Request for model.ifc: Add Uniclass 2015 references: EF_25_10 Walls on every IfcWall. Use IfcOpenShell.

First a look at what the model holds.

```python
import ifcopenshell

model = ifcopenshell.open("model.ifc")
print(model.schema)
print("classifications:", [c.Name for c in model.by_type("IfcClassification")])
for ifc_class in ("IfcDoor", "IfcRoof", "IfcStair", "IfcWall", "IfcWindow"):
    print(ifc_class, len(model.by_type(ifc_class)))
```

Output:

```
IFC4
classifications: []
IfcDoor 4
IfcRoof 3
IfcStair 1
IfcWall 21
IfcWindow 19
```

```python
import ifcopenshell
import ifcopenshell.api.classification

model = ifcopenshell.open("model.ifc")

system = ifcopenshell.api.classification.add_classification(model, classification="Uniclass 2015")

codes = {
    "IfcWall": ("EF_25_10", "Walls"),
}
for ifc_class, (code, name) in codes.items():
    products = model.by_type(ifc_class)
    ifcopenshell.api.classification.add_reference(
        model, products=products, classification=system, identification=code, name=name
    )
    print(code, len(products))

model.write("model_updated.ifc")
```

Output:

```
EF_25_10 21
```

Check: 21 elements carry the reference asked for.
